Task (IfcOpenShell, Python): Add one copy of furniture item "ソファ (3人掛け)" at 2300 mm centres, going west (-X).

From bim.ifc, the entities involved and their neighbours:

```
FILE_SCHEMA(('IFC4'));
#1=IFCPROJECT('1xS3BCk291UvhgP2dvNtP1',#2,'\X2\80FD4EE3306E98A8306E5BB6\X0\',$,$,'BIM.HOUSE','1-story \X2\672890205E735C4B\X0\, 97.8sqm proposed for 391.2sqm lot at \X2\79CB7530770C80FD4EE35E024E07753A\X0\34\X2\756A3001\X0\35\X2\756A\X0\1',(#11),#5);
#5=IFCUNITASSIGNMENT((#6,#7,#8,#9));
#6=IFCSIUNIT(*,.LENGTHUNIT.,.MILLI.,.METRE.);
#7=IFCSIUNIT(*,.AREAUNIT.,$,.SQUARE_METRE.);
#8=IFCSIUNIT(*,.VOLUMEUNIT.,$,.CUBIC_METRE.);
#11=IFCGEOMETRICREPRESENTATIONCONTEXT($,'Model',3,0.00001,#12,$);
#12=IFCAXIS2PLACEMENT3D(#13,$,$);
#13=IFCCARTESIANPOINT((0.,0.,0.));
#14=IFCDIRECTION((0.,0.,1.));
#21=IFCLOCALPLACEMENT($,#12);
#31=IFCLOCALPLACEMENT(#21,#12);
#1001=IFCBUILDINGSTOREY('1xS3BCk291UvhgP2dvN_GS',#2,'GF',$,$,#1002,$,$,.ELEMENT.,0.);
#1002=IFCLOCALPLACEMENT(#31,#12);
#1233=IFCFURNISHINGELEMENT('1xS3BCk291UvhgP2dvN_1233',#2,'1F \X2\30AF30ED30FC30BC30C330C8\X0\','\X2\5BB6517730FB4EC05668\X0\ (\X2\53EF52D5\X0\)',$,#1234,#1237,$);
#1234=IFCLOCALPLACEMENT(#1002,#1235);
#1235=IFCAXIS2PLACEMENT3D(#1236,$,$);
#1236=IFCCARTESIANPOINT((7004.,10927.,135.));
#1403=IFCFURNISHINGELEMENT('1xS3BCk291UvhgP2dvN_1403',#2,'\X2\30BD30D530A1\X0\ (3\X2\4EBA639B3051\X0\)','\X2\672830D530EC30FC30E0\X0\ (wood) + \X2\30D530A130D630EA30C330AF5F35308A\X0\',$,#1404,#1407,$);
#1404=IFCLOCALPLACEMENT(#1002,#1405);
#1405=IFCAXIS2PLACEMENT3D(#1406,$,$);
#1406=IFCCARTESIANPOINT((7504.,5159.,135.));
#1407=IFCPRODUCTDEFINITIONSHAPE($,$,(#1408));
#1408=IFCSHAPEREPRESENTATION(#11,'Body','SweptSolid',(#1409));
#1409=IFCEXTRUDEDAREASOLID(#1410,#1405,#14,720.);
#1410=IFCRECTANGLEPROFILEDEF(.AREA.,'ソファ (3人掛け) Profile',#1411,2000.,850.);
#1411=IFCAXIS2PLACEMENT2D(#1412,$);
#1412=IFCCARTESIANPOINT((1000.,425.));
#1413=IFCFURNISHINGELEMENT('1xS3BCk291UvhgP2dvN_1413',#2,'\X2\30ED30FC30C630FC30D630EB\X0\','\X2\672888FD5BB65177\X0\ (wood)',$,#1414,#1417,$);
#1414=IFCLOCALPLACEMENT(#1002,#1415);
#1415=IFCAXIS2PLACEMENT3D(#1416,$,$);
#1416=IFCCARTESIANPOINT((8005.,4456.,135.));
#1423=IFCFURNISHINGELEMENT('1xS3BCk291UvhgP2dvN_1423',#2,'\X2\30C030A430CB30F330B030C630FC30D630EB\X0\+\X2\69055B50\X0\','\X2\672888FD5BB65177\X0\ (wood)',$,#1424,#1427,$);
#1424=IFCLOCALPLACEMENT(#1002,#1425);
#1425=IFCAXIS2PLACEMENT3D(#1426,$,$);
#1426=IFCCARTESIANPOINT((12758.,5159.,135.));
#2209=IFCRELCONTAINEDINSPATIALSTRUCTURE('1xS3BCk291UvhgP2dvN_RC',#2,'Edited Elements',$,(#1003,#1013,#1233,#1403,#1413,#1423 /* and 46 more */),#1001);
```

```python
import numpy as np
import ifcopenshell
import ifcopenshell.api.geometry
import ifcopenshell.api.root
import ifcopenshell.util.element
import ifcopenshell.util.placement

model = ifcopenshell.open("bim.ifc")


def reuse_history(source, copy):
    """copy_class also copies each property set's owner history, people and application; keep the originals."""
    for rel in copy.IsDefinedBy:
        if rel.is_a("IfcRelDefinesByProperties") and (history := rel.RelatingPropertyDefinition.OwnerHistory):
            rel.RelatingPropertyDefinition.OwnerHistory = source.OwnerHistory
            ifcopenshell.util.element.remove_deep2(model, history)


source = model.by_id(1403)
base = ifcopenshell.util.placement.get_local_placement(source.ObjectPlacement)
step = np.array([-1.0, 0.0, 0.0]) * 2300.0

for i in range(1, 2):
    copy = ifcopenshell.api.root.copy_class(model, product=source)
    copy.Representation = ifcopenshell.util.element.copy_deep(
        model, source.Representation, exclude=["IfcGeometricRepresentationContext", "IfcRepresentationMap"]
    )
    reuse_history(source, copy)
    matrix = base.copy()
    matrix[:3, 3] += i * step
    print("added at", matrix[:3, 3].round(3) + 0.0)
    ifcopenshell.api.geometry.edit_object_placement(model, product=copy, matrix=matrix, is_si=False)

model.write("bim_updated.ifc")
```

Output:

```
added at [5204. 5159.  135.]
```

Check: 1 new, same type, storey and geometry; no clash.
